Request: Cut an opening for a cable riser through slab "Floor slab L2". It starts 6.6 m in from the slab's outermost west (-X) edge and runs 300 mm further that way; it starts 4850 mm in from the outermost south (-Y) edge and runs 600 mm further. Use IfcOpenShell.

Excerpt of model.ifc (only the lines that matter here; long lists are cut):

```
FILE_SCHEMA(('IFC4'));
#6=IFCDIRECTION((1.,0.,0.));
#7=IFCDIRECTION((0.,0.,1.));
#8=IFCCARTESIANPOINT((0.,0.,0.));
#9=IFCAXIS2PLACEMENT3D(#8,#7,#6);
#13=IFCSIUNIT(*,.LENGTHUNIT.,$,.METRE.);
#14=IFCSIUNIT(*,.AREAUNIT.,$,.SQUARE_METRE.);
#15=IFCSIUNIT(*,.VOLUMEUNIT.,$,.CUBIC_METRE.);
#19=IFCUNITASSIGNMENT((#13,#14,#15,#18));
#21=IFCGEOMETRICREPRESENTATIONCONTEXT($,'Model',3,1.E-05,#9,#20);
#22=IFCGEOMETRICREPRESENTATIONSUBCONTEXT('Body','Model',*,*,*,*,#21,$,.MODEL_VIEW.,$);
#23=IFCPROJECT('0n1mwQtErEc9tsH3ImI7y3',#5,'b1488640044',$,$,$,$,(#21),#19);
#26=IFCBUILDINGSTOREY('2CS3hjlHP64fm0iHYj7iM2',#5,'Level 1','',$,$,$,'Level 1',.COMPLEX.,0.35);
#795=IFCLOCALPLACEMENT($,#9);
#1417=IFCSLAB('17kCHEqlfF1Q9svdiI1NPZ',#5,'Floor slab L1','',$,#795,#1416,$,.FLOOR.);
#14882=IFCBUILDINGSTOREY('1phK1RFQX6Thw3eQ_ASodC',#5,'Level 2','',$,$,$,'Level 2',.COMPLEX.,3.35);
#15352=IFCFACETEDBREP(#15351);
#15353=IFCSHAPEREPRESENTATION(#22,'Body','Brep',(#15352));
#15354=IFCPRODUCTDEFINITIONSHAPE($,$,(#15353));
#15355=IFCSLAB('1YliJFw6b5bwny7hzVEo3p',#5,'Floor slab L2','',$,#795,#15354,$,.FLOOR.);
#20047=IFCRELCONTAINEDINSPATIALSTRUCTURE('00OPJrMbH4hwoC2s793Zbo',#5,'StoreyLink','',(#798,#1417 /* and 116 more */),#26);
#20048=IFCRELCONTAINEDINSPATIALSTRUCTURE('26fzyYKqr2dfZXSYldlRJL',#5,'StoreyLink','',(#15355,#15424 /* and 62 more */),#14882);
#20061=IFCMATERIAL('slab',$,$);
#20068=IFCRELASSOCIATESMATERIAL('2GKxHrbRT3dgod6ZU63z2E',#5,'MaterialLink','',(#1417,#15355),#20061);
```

```python
import numpy as np
import ifcopenshell
import ifcopenshell.api.feature
import ifcopenshell.api.geometry
import ifcopenshell.api.root
import ifcopenshell.geom
import ifcopenshell.util.placement
import ifcopenshell.util.representation
import ifcopenshell.util.shape
import ifcopenshell.util.unit

model = ifcopenshell.open("model.ifc")
unit_scale = ifcopenshell.util.unit.calculate_unit_scale(model)
settings = ifcopenshell.geom.settings()


def volume(element):
    """Net volume in cubic metres, openings subtracted."""
    shape = ifcopenshell.geom.create_shape(settings, element)
    return ifcopenshell.util.shape.get_volume(shape.geometry)


slab = model.by_guid("1YliJFw6b5bwny7hzVEo3p")
before = volume(slab)

# Extent in the slab's own axes, in metres. The edges named are its -X and -Y sides.
slab_shape = ifcopenshell.geom.create_shape(settings, slab)
vertices = ifcopenshell.util.shape.get_vertices(slab_shape.geometry)
x_min, y_min, bottom = vertices.min(axis=0)
top = vertices[:, 2].max()

opening = ifcopenshell.api.root.create_entity(model, ifc_class="IfcOpeningElement", name="Cable riser opening", predefined_type="OPENING")
context = ifcopenshell.util.representation.get_context(model, "Model", "Body", "MODEL_VIEW")
width, depth = 0.3, 0.6
outline = [(0.0, 0.0), (width, 0.0), (width, depth), (0.0, depth), (0.0, 0.0)]
# Overshoot both faces by 50 mm so the cut is clean.
shape = ifcopenshell.api.geometry.add_slab_representation(
    model, context=context, depth=top - bottom + 0.1, polyline=outline
)
ifcopenshell.api.geometry.assign_representation(model, product=opening, representation=shape)

matrix = ifcopenshell.util.placement.get_local_placement(slab.ObjectPlacement)
matrix[:, 3] = matrix @ np.append(np.array([x_min + 6.6, y_min + 4.85, bottom - 0.05]) / unit_scale, 1.0)
ifcopenshell.api.geometry.edit_object_placement(model, product=opening, matrix=matrix, is_si=False)
ifcopenshell.api.feature.add_feature(model, feature=opening, element=slab)

after = volume(slab)

print(f"slab volume {before:.3f} -> {after:.3f} m3")

model.write("model_edited.ifc")
```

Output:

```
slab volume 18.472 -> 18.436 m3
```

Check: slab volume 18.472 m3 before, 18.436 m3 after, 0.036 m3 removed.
